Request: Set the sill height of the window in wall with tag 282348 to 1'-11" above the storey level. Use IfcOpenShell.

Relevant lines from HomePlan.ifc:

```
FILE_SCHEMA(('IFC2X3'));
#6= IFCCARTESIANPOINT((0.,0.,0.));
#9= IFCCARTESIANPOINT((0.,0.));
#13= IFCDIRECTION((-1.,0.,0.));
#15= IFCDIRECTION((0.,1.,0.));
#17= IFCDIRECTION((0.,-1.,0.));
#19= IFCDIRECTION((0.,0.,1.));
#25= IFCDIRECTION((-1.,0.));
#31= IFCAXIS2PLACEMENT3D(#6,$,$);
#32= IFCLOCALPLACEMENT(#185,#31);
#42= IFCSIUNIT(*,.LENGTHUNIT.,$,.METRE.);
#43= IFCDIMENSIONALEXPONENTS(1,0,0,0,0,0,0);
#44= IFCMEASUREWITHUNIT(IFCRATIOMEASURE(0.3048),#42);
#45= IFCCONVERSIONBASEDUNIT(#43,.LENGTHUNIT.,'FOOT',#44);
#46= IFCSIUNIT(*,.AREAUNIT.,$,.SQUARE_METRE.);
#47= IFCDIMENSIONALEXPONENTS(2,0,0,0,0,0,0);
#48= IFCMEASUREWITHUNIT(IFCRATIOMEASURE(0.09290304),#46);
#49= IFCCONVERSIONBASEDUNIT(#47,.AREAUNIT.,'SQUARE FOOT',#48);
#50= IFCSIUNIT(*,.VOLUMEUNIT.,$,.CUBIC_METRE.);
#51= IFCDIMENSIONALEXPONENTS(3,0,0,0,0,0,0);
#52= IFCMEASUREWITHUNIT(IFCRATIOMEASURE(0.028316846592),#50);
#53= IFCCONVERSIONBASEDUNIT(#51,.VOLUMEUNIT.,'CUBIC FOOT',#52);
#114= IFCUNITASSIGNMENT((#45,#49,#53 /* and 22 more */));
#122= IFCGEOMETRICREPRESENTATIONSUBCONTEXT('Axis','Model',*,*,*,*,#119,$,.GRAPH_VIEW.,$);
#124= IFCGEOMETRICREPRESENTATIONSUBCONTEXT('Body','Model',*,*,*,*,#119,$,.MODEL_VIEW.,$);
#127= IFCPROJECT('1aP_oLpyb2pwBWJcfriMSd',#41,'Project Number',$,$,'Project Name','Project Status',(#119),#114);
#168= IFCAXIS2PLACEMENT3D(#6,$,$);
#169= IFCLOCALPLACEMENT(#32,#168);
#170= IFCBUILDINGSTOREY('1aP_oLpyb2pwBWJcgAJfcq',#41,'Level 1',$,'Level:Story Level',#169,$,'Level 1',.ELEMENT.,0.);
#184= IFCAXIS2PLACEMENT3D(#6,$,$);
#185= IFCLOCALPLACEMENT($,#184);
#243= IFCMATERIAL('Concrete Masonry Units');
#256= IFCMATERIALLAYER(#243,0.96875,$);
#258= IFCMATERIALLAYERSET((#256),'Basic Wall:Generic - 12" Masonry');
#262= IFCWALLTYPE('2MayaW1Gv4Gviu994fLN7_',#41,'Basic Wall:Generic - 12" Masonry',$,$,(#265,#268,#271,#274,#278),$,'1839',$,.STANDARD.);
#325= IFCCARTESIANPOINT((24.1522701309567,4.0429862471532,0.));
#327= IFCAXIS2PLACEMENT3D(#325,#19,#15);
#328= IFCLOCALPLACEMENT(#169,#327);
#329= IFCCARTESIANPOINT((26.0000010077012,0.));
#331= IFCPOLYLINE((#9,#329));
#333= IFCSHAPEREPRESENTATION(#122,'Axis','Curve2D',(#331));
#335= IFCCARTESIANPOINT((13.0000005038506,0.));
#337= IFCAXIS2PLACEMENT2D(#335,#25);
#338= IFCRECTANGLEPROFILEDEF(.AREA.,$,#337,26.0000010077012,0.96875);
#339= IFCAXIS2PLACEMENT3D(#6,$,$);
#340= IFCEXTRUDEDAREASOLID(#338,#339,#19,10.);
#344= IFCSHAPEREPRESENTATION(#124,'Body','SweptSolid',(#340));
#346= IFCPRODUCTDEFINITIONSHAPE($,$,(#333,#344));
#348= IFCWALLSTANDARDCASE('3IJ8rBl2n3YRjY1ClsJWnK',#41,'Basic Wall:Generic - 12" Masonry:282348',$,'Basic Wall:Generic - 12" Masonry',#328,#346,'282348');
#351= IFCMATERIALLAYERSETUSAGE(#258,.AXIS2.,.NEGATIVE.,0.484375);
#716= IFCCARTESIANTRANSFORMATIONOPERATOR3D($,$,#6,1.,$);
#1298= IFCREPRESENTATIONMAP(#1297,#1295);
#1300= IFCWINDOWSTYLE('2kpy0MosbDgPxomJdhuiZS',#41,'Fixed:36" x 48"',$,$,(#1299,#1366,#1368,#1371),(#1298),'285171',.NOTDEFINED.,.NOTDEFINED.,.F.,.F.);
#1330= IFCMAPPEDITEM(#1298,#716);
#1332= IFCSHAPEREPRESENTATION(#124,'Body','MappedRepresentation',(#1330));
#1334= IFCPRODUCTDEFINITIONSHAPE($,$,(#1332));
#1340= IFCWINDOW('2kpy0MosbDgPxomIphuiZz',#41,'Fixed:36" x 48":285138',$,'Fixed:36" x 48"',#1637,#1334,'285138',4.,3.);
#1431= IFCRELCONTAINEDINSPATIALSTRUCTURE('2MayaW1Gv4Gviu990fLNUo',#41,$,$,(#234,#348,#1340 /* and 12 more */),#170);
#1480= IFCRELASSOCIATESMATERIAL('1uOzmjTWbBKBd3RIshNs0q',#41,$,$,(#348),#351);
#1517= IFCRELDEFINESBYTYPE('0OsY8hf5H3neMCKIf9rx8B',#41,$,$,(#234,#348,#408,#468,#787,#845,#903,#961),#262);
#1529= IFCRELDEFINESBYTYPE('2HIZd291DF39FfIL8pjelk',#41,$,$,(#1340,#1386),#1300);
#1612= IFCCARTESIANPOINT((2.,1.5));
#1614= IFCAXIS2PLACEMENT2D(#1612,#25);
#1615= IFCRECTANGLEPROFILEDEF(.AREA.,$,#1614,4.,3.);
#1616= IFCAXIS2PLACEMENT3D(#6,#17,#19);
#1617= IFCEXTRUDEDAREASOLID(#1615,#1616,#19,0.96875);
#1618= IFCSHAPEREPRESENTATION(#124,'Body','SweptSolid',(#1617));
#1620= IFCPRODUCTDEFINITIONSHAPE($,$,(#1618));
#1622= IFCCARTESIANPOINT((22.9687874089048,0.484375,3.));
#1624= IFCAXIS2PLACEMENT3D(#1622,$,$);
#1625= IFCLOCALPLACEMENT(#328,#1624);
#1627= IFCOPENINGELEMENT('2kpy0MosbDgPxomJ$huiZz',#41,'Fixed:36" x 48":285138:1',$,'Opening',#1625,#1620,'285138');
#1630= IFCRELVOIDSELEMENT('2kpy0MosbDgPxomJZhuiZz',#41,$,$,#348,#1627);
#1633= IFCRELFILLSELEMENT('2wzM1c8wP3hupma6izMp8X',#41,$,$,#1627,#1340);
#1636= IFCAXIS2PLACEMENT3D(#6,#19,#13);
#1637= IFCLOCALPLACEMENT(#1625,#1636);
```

```python
import numpy as np
import ifcopenshell
import ifcopenshell.api.geometry
import ifcopenshell.geom
import ifcopenshell.util.element
import ifcopenshell.util.placement
import ifcopenshell.util.shape
import ifcopenshell.util.unit

model = ifcopenshell.open("HomePlan.ifc")
unit_scale = ifcopenshell.util.unit.calculate_unit_scale(model)

window = model.by_guid("2kpy0MosbDgPxomIphuiZz")
opening = window.FillsVoids[0].RelatingOpeningElement
storey = ifcopenshell.util.element.get_container(window, ifc_class="IfcBuildingStorey")
level = ifcopenshell.util.placement.get_local_placement(storey.ObjectPlacement)[2, 3]

# The opening's origin need not be at the sill, so measure its lowest point.
shape = ifcopenshell.geom.create_shape(ifcopenshell.geom.settings(), opening)
bottom = ifcopenshell.util.shape.get_shape_bottom_elevation(shape, shape.geometry) / unit_scale
dz = level + 23 * 0.0254 / unit_scale - bottom

shift = np.array([0.0, 0.0, dz])
# The window is placed relative to its opening, so it follows when the opening moves.
matrix = ifcopenshell.util.placement.get_local_placement(opening.ObjectPlacement)
matrix[:3, 3] += shift
ifcopenshell.api.geometry.edit_object_placement(
    model, product=opening, matrix=matrix, is_si=False, should_transform_children=True
)

print(f"moved by {dz * unit_scale:+.3f} m")

model.write("HomePlan_edited.ifc")
```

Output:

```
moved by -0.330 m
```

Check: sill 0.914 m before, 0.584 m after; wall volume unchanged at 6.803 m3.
